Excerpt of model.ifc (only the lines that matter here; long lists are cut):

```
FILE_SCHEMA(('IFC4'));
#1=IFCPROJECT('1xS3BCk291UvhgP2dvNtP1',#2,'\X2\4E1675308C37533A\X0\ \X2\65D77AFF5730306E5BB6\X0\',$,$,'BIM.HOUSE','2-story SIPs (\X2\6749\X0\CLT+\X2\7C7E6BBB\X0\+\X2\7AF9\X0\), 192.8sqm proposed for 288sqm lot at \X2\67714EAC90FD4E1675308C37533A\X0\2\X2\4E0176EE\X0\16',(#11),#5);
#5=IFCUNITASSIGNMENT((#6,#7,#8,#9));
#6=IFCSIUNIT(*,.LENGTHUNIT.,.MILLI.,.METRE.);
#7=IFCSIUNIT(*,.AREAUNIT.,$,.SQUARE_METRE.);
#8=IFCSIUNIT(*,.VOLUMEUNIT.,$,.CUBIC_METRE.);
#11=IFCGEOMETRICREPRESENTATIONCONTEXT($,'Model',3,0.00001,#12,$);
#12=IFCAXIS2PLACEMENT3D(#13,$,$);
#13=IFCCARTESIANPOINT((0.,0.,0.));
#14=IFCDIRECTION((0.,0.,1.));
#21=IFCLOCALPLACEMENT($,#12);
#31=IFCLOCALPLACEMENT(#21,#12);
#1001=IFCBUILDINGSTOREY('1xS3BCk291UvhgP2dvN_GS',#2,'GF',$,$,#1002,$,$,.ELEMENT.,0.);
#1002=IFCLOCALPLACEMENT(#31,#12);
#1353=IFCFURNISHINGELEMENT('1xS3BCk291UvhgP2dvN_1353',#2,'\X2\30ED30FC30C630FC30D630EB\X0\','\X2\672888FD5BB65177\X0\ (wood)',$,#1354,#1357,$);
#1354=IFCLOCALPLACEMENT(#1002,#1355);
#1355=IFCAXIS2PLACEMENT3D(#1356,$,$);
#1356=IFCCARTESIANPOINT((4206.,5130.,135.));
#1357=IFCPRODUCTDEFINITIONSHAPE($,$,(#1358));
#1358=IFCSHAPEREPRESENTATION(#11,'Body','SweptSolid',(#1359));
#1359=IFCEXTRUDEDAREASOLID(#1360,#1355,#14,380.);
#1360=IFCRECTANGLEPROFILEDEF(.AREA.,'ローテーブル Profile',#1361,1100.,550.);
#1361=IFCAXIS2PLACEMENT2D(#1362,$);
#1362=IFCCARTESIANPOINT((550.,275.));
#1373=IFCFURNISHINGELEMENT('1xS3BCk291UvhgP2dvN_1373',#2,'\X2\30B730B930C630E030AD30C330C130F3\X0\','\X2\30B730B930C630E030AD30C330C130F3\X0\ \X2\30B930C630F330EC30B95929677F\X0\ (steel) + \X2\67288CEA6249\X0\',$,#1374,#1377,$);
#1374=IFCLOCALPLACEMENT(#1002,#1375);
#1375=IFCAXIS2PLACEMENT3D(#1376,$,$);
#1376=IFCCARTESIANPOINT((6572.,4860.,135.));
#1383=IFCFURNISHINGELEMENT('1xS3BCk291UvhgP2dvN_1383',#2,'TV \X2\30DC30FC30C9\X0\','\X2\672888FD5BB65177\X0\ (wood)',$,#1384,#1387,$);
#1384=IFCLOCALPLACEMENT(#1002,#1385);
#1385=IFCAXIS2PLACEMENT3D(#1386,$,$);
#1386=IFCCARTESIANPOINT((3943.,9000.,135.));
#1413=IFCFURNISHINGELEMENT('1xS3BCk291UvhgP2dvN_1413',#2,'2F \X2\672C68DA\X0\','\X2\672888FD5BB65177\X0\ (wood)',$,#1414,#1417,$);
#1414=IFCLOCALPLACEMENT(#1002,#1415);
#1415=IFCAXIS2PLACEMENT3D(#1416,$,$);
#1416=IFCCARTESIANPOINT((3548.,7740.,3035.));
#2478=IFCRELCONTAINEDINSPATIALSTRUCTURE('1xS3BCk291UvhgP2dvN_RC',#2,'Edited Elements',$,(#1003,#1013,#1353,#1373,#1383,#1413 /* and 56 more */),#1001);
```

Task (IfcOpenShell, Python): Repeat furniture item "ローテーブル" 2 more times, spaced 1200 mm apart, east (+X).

```python
import numpy as np
import ifcopenshell
import ifcopenshell.api.geometry
import ifcopenshell.api.root
import ifcopenshell.util.element
import ifcopenshell.util.placement

model = ifcopenshell.open("model.ifc")


def reuse_history(source, copy):
    """copy_class also copies each property set's owner history, people and application; keep the originals."""
    for rel in copy.IsDefinedBy:
        if rel.is_a("IfcRelDefinesByProperties") and (history := rel.RelatingPropertyDefinition.OwnerHistory):
            rel.RelatingPropertyDefinition.OwnerHistory = source.OwnerHistory
            ifcopenshell.util.element.remove_deep2(model, history)


source = model.by_id(1353)
base = ifcopenshell.util.placement.get_local_placement(source.ObjectPlacement)
step = np.array([1.0, 0.0, 0.0]) * 1200.0

for i in range(1, 3):
    copy = ifcopenshell.api.root.copy_class(model, product=source)
    copy.Representation = ifcopenshell.util.element.copy_deep(
        model, source.Representation, exclude=["IfcGeometricRepresentationContext", "IfcRepresentationMap"]
    )
    reuse_history(source, copy)
    matrix = base.copy()
    matrix[:3, 3] += i * step
    print("added at", matrix[:3, 3].round(3) + 0.0)
    ifcopenshell.api.geometry.edit_object_placement(model, product=copy, matrix=matrix, is_si=False)

model.write("model_v2.ifc")
```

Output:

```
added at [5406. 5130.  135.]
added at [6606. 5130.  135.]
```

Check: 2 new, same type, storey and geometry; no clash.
